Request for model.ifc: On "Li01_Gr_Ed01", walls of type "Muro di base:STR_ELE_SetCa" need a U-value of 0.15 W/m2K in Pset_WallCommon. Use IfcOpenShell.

First a look at what the model holds.

```python
import ifcopenshell
import ifcopenshell.util.element

model = ifcopenshell.open("model.ifc")
print(model.schema)
storey = next(s for s in model.by_type("IfcBuildingStorey") if s.Name == "Li01_Gr_Ed01")
walls = [e for e in ifcopenshell.util.element.get_decomposition(storey) if e.is_a("IfcWall")]
seen = {}
for e in walls:
    element_type = ifcopenshell.util.element.get_type(e)
    key = (element_type.Name if element_type != e and element_type else None, ifcopenshell.util.element.get_pset(e, "Pset_WallCommon", "ThermalTransmittance"))
    seen[key] = seen.get(key, 0) + 1
for (name, value), count in sorted(seen.items(), key=str):
    print(count, "x", name, "|", value)
```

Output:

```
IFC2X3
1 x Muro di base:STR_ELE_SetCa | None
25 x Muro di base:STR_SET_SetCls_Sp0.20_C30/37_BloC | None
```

```python
import ifcopenshell
import ifcopenshell.api.pset
import ifcopenshell.util.element

model = ifcopenshell.open("model.ifc")

storey = next(s for s in model.by_type("IfcBuildingStorey") if s.Name == "Li01_Gr_Ed01")
walls = [e for e in ifcopenshell.util.element.get_decomposition(storey) if e.is_a("IfcWall")]

count = 0
for e in walls:
    element_type = ifcopenshell.util.element.get_type(e)
    if element_type in (None, e) or element_type.Name != "Muro di base:STR_ELE_SetCa":
        continue
    # add_pset returns the element's existing set when there is one.
    pset = ifcopenshell.api.pset.add_pset(model, product=e, name="Pset_WallCommon")
    ifcopenshell.api.pset.edit_pset(model, pset=pset, properties={"ThermalTransmittance": 0.15})
    count += 1

print(count, "walls updated")

model.write("model_edited.ifc")
```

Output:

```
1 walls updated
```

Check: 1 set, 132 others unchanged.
